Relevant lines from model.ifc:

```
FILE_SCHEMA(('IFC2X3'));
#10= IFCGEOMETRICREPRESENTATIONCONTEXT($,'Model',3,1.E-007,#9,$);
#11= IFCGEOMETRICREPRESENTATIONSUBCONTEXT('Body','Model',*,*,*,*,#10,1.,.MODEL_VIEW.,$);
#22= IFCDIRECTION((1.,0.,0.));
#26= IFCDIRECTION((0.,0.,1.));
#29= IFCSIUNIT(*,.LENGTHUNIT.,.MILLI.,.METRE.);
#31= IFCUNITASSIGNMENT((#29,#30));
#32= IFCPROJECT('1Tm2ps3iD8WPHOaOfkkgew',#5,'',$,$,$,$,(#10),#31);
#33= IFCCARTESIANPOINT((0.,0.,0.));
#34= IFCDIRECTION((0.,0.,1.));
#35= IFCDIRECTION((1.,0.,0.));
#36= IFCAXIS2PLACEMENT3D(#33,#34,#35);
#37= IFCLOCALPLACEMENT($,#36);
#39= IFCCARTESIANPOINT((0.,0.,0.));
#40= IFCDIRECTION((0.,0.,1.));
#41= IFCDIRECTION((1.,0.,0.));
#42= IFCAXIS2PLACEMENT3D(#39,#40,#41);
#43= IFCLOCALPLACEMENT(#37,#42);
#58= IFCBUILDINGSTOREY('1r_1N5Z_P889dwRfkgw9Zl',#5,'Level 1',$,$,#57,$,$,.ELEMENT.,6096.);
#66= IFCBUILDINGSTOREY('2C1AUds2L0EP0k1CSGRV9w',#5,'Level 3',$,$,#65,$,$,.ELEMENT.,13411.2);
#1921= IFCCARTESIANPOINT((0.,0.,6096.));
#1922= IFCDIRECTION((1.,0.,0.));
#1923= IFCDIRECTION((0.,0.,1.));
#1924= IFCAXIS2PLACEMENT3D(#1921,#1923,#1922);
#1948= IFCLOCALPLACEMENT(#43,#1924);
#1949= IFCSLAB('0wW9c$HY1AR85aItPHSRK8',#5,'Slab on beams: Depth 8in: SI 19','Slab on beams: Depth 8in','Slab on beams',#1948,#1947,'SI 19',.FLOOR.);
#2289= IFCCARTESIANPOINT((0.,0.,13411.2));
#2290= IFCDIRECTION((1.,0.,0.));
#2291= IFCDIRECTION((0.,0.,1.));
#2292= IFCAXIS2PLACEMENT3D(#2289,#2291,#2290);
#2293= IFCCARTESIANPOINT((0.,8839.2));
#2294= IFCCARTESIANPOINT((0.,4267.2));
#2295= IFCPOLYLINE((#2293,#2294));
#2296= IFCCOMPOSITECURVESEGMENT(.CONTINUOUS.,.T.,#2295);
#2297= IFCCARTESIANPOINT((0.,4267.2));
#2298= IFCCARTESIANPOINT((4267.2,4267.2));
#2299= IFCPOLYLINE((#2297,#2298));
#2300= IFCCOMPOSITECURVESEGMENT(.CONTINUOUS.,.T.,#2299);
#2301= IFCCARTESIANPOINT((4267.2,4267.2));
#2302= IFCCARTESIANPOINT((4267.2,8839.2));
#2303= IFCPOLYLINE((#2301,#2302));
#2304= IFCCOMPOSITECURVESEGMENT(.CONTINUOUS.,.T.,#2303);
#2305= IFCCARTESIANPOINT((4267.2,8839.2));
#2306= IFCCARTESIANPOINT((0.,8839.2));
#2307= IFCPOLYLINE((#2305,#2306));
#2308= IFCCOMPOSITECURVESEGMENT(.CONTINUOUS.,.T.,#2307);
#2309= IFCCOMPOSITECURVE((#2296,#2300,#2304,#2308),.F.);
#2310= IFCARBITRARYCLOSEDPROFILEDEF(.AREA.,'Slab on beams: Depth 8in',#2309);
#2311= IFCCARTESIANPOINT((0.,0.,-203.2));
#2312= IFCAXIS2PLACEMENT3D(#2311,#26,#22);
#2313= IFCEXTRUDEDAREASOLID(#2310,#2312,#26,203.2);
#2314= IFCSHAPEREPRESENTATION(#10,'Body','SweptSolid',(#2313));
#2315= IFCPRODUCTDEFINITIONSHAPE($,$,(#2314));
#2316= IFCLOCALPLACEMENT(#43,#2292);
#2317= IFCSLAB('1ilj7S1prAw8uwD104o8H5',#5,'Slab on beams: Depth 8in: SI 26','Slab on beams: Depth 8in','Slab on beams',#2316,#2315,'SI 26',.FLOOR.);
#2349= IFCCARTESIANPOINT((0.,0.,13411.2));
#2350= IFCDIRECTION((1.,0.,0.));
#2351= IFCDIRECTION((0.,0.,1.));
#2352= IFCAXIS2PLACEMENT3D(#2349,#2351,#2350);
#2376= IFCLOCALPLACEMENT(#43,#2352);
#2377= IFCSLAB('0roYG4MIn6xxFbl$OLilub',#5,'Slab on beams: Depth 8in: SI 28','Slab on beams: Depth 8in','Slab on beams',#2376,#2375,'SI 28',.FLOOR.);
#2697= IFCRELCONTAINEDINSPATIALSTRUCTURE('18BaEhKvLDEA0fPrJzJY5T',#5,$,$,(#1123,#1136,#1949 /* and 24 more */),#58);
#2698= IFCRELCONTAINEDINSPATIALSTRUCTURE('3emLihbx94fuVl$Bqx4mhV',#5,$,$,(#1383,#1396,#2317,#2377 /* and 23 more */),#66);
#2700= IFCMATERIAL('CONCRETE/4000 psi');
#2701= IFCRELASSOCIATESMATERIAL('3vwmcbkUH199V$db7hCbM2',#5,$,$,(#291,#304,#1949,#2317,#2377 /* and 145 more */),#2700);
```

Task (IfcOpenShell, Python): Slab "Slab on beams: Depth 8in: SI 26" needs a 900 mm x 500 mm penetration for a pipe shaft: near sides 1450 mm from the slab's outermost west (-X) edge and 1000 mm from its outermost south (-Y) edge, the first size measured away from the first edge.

```python
import numpy as np
import ifcopenshell
import ifcopenshell.api.feature
import ifcopenshell.api.geometry
import ifcopenshell.api.root
import ifcopenshell.geom
import ifcopenshell.util.placement
import ifcopenshell.util.representation
import ifcopenshell.util.shape
import ifcopenshell.util.unit

model = ifcopenshell.open("model.ifc")
unit_scale = ifcopenshell.util.unit.calculate_unit_scale(model)
settings = ifcopenshell.geom.settings()


def volume(element):
    """Net volume in cubic metres, openings subtracted."""
    shape = ifcopenshell.geom.create_shape(settings, element)
    return ifcopenshell.util.shape.get_volume(shape.geometry)


slab = model.by_id(2317)
before = volume(slab)

# Extent in the slab's own axes, in metres. The edges named are its -X and -Y sides.
slab_shape = ifcopenshell.geom.create_shape(settings, slab)
vertices = ifcopenshell.util.shape.get_vertices(slab_shape.geometry)
x_min, y_min, bottom = vertices.min(axis=0)
top = vertices[:, 2].max()

opening = ifcopenshell.api.root.create_entity(model, ifc_class="IfcOpeningElement", name="Pipe shaft opening")
context = ifcopenshell.util.representation.get_context(model, "Model", "Body", "MODEL_VIEW")
width, depth = 0.9, 0.5
outline = [(0.0, 0.0), (width, 0.0), (width, depth), (0.0, depth), (0.0, 0.0)]
# Overshoot both faces by 50 mm so the cut is clean.
shape = ifcopenshell.api.geometry.add_slab_representation(
    model, context=context, depth=top - bottom + 0.1, polyline=outline
)
ifcopenshell.api.geometry.assign_representation(model, product=opening, representation=shape)

matrix = ifcopenshell.util.placement.get_local_placement(slab.ObjectPlacement)
matrix[:, 3] = matrix @ np.append(np.array([x_min + 1.45, y_min + 1, bottom - 0.05]) / unit_scale, 1.0)
ifcopenshell.api.geometry.edit_object_placement(model, product=opening, matrix=matrix, is_si=False)
ifcopenshell.api.feature.add_feature(model, feature=opening, element=slab)

after = volume(slab)

print(f"slab volume {before:.3f} -> {after:.3f} m3")

model.write("model_edited.ifc")
```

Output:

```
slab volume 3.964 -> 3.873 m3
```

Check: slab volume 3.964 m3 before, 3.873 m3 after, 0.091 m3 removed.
